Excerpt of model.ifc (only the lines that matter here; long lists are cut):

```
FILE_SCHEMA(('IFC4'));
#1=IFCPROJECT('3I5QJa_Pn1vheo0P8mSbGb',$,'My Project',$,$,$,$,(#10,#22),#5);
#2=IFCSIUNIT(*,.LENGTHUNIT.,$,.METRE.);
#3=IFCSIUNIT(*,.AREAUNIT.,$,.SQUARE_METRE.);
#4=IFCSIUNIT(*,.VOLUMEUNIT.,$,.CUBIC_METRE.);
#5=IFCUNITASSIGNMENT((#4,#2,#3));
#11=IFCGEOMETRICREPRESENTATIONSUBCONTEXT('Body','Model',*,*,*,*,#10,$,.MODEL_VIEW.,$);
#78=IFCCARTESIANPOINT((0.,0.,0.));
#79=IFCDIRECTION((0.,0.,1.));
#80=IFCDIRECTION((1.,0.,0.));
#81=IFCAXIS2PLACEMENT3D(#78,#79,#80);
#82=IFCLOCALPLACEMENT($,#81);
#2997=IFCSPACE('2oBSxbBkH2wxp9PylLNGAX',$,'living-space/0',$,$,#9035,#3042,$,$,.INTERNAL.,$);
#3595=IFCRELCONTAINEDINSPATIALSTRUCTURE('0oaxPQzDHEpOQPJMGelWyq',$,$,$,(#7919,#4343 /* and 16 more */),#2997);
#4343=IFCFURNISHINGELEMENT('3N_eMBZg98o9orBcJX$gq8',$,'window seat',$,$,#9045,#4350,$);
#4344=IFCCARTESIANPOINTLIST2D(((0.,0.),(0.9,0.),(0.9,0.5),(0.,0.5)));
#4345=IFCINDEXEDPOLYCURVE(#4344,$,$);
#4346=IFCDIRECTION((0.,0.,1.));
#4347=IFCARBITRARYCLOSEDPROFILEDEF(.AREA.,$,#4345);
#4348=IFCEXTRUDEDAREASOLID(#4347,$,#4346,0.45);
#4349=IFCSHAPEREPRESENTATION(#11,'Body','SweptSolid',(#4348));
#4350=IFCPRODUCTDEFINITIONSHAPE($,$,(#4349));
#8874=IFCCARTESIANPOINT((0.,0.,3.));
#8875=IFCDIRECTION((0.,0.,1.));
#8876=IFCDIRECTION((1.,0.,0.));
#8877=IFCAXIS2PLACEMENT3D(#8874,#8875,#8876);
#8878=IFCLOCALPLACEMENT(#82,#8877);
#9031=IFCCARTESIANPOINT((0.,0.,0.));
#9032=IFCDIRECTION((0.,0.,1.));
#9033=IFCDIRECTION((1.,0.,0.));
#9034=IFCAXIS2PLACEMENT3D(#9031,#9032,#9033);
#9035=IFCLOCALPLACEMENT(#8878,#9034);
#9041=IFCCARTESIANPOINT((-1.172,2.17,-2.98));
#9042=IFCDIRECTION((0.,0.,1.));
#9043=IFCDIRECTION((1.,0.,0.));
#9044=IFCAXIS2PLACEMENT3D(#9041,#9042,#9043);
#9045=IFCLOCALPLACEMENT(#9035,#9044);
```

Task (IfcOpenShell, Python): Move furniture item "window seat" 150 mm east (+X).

```python
import ifcopenshell
import ifcopenshell.api.geometry
import ifcopenshell.util.placement
import ifcopenshell.util.unit

model = ifcopenshell.open("model.ifc")
unit_scale = ifcopenshell.util.unit.calculate_unit_scale(model)

item = model.by_id(4343)
matrix = ifcopenshell.util.placement.get_local_placement(item.ObjectPlacement)
matrix[0, 3] += 0.15 / unit_scale
ifcopenshell.api.geometry.edit_object_placement(model, product=item, matrix=matrix, is_si=False)

print(ifcopenshell.util.placement.get_local_placement(item.ObjectPlacement).round(3) + 0.0)

model.write("model-out.ifc")
```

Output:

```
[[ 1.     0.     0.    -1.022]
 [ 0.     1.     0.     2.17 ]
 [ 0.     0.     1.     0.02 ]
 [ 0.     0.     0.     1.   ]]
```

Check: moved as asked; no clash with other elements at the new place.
